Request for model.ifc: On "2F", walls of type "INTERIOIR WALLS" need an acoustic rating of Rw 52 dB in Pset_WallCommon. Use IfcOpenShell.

First a look at what the model holds.

```python
import ifcopenshell
import ifcopenshell.util.element

model = ifcopenshell.open("model.ifc")
print(model.schema)
storey = next(s for s in model.by_type("IfcBuildingStorey") if s.Name == "2F")
walls = [e for e in ifcopenshell.util.element.get_decomposition(storey) if e.is_a("IfcWall")]
seen = {}
for e in walls:
    element_type = ifcopenshell.util.element.get_type(e)
    key = (element_type.Name if element_type != e and element_type else None, ifcopenshell.util.element.get_pset(e, "Pset_WallCommon", "AcousticRating"))
    seen[key] = seen.get(key, 0) + 1
for (name, value), count in sorted(seen.items(), key=str):
    print(count, "x", name, "|", value)
```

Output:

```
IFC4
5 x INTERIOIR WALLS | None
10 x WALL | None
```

```python
import ifcopenshell
import ifcopenshell.api.pset
import ifcopenshell.util.element

model = ifcopenshell.open("model.ifc")

storey = next(s for s in model.by_type("IfcBuildingStorey") if s.Name == "2F")
walls = [e for e in ifcopenshell.util.element.get_decomposition(storey) if e.is_a("IfcWall")]

count = 0
for e in walls:
    element_type = ifcopenshell.util.element.get_type(e)
    if element_type in (None, e) or element_type.Name != "INTERIOIR WALLS":
        continue
    # add_pset returns the element's existing set when there is one.
    pset = ifcopenshell.api.pset.add_pset(model, product=e, name="Pset_WallCommon")
    ifcopenshell.api.pset.edit_pset(model, pset=pset, properties={"AcousticRating": "Rw 52 dB"})
    count += 1

print(count, "walls updated")

model.write("model_v2.ifc")
```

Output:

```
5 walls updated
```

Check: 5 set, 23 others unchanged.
